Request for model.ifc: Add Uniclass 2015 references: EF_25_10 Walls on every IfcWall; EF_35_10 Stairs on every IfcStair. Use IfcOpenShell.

First a look at what the model holds.

```python
import ifcopenshell

model = ifcopenshell.open("model.ifc")
print(model.schema)
print("classifications:", [c.Name for c in model.by_type("IfcClassification")])
for ifc_class in ("IfcDoor", "IfcRoof", "IfcStair", "IfcWall", "IfcWindow"):
    print(ifc_class, len(model.by_type(ifc_class)))
```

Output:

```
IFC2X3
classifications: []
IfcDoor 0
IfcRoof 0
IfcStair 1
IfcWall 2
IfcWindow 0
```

```python
import ifcopenshell
import ifcopenshell.api.classification

model = ifcopenshell.open("model.ifc")

# IFC2X3 requires Source and Edition and has no link from the project to the system.
system = model.create_entity("IfcClassification", Source="NBS", Edition="2015", Name="Uniclass 2015")

codes = {
    "IfcWall": ("EF_25_10", "Walls"),
    "IfcStair": ("EF_35_10", "Stairs"),
}
for ifc_class, (code, name) in codes.items():
    products = model.by_type(ifc_class)
    ifcopenshell.api.classification.add_reference(
        model, products=products, classification=system, identification=code, name=name
    )
    print(code, len(products))

model.write("model_updated.ifc")
```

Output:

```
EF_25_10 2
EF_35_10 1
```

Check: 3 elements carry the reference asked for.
